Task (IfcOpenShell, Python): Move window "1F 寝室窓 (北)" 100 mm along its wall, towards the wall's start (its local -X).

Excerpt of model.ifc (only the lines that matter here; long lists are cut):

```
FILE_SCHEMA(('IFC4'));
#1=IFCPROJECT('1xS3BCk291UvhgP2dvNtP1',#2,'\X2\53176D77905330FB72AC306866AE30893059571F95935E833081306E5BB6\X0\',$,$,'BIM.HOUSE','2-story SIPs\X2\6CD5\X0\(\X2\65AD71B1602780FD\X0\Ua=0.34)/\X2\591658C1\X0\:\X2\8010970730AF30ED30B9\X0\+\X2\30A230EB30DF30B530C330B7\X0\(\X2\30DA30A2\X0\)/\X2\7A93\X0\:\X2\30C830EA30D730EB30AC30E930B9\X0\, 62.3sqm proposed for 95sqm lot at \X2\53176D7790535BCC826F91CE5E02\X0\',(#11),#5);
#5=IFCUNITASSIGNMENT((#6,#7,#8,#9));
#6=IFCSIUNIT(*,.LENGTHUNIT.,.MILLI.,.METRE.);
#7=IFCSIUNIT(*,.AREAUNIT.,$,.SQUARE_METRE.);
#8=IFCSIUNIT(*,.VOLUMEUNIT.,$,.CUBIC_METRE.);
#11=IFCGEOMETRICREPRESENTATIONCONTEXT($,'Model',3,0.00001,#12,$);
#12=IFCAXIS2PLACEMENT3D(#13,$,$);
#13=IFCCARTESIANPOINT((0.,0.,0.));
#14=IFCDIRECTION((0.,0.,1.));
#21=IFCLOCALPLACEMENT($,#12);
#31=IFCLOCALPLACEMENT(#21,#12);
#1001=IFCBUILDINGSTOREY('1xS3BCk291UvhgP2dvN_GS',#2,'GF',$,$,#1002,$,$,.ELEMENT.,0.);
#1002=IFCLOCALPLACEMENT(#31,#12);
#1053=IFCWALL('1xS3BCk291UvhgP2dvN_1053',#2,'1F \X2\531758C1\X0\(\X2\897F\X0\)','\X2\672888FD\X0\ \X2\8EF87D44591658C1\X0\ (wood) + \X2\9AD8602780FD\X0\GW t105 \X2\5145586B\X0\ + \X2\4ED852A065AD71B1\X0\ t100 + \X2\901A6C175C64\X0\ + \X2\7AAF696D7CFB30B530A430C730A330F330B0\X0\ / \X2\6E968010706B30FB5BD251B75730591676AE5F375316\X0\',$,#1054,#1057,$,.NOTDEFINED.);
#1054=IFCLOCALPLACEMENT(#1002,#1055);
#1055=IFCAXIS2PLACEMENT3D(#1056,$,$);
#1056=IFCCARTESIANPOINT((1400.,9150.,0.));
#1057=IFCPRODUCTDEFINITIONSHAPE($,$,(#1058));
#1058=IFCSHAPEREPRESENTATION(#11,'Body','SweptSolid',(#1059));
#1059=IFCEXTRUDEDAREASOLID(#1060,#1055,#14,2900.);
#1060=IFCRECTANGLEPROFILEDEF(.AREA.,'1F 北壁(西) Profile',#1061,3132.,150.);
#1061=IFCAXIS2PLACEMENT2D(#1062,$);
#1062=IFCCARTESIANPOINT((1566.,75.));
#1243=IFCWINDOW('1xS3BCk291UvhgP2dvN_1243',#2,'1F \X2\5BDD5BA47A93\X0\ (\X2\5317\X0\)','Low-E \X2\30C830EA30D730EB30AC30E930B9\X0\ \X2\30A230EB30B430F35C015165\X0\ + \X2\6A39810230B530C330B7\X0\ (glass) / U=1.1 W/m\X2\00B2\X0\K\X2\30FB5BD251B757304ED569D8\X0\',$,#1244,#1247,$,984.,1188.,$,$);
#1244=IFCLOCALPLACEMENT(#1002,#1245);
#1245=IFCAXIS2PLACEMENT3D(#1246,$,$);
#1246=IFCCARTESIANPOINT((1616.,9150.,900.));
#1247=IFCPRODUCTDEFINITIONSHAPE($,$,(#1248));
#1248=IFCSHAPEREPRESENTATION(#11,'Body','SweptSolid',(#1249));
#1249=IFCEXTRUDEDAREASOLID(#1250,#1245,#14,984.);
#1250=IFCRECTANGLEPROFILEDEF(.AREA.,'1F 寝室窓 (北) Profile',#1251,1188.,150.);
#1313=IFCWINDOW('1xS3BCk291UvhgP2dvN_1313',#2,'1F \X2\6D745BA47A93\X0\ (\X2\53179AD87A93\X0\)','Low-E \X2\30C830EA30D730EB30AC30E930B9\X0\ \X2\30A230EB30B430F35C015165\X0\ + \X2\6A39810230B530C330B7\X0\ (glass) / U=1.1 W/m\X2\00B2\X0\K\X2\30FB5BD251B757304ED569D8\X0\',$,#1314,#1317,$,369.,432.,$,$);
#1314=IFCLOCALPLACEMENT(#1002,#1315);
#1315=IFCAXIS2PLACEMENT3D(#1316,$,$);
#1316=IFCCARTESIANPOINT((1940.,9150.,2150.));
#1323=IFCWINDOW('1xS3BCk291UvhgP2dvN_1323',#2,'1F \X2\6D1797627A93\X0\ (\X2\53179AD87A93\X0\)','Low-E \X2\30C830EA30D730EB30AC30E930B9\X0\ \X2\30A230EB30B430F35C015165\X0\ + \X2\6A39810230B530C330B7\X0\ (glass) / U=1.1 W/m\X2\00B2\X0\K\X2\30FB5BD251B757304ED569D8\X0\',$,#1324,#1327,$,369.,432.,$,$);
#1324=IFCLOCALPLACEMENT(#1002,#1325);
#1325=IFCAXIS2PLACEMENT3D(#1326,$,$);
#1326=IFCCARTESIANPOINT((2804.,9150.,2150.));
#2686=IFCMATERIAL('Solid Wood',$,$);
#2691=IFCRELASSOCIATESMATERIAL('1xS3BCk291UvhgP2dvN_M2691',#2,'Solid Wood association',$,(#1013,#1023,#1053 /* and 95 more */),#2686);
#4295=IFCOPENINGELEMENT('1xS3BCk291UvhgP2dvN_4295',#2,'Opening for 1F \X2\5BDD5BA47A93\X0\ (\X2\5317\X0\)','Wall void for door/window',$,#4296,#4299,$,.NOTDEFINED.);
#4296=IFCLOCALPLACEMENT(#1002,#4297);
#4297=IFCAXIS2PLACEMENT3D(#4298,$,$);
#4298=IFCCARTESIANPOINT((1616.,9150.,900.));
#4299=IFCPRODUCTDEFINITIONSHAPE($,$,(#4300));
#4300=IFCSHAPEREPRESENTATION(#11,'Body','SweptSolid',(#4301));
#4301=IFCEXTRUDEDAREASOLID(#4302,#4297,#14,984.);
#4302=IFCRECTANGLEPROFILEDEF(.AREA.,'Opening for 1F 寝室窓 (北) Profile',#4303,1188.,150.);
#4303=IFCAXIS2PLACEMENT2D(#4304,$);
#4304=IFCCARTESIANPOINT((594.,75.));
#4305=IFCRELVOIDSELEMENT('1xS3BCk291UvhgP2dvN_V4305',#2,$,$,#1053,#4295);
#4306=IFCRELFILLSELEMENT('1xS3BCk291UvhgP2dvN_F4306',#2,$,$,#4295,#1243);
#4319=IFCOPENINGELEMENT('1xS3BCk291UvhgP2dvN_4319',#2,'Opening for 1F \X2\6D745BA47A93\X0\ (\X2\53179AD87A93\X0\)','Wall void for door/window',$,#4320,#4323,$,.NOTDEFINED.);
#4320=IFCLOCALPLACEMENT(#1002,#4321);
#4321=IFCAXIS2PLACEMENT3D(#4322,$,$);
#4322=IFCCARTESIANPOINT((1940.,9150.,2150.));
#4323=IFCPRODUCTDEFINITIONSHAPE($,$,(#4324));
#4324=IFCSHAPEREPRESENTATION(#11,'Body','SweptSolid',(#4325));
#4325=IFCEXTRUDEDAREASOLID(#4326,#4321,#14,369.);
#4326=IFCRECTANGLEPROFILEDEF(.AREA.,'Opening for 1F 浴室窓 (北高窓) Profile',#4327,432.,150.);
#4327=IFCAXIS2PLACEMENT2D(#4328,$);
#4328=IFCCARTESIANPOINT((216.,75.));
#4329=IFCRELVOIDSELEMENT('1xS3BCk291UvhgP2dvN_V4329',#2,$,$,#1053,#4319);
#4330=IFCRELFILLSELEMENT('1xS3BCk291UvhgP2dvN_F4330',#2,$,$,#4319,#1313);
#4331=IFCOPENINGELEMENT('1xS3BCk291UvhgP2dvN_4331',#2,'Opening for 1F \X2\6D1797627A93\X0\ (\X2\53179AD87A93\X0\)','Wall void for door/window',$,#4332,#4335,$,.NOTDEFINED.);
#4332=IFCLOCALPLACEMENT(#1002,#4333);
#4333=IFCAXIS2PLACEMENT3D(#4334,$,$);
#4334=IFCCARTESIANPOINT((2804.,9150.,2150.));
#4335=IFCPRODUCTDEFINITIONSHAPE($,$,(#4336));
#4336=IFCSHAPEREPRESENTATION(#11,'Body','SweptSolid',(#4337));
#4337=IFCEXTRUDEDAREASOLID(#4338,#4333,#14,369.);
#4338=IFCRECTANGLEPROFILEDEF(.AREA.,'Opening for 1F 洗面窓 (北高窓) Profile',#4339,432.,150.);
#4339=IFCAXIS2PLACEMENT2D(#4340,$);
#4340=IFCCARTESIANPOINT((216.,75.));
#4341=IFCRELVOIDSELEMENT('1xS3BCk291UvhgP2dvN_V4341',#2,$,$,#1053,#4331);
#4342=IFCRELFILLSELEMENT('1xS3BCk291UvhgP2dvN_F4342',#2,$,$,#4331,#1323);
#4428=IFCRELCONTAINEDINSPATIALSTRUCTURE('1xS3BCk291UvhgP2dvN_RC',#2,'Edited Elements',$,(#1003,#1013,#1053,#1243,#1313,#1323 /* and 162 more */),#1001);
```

```python
import ifcopenshell
import ifcopenshell.api.geometry
import ifcopenshell.util.placement
import ifcopenshell.util.unit

model = ifcopenshell.open("model.ifc")
unit_scale = ifcopenshell.util.unit.calculate_unit_scale(model)

window = model.by_id(1243)
opening = window.FillsVoids[0].RelatingOpeningElement
wall = opening.VoidsElements[0].RelatingBuildingElement

wall_matrix = ifcopenshell.util.placement.get_local_placement(wall.ObjectPlacement)
shift = wall_matrix[:3, 0] * -0.1 / unit_scale
before = ifcopenshell.util.placement.get_local_placement(window.ObjectPlacement)[:3, 3].copy()

# The window is not placed relative to its opening, so move both.
for product in (opening, window):
    matrix = ifcopenshell.util.placement.get_local_placement(product.ObjectPlacement)
    matrix[:3, 3] += shift
    ifcopenshell.api.geometry.edit_object_placement(model, product=product, matrix=matrix, is_si=False)

after = ifcopenshell.util.placement.get_local_placement(window.ObjectPlacement)[:3, 3]
print("window moved by", (after - before).round(3) + 0.0)

model.write("model-out.ifc")
```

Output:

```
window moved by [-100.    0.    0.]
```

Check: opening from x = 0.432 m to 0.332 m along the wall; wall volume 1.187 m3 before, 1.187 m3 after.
